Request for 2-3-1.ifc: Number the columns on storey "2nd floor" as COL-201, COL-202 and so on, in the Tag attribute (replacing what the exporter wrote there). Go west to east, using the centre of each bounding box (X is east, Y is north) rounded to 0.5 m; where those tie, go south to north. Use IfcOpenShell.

First a look at what the model holds.

```python
import ifcopenshell
import ifcopenshell.util.element
import ifcopenshell.util.placement

model = ifcopenshell.open("2-3-1.ifc")
print(model.schema)
storey = next(s for s in model.by_type("IfcBuildingStorey") if s.Name == "2nd floor")
columns = [e for e in ifcopenshell.util.element.get_decomposition(storey) if e.is_a("IfcColumn")]
for e in sorted(columns, key=lambda e: e.id()):
    origin = ifcopenshell.util.placement.get_local_placement(e.ObjectPlacement)[:3, 3]
    print(e.id(), e.Tag, e.Name, origin.round(2) + 0.0, sep=" | ")
```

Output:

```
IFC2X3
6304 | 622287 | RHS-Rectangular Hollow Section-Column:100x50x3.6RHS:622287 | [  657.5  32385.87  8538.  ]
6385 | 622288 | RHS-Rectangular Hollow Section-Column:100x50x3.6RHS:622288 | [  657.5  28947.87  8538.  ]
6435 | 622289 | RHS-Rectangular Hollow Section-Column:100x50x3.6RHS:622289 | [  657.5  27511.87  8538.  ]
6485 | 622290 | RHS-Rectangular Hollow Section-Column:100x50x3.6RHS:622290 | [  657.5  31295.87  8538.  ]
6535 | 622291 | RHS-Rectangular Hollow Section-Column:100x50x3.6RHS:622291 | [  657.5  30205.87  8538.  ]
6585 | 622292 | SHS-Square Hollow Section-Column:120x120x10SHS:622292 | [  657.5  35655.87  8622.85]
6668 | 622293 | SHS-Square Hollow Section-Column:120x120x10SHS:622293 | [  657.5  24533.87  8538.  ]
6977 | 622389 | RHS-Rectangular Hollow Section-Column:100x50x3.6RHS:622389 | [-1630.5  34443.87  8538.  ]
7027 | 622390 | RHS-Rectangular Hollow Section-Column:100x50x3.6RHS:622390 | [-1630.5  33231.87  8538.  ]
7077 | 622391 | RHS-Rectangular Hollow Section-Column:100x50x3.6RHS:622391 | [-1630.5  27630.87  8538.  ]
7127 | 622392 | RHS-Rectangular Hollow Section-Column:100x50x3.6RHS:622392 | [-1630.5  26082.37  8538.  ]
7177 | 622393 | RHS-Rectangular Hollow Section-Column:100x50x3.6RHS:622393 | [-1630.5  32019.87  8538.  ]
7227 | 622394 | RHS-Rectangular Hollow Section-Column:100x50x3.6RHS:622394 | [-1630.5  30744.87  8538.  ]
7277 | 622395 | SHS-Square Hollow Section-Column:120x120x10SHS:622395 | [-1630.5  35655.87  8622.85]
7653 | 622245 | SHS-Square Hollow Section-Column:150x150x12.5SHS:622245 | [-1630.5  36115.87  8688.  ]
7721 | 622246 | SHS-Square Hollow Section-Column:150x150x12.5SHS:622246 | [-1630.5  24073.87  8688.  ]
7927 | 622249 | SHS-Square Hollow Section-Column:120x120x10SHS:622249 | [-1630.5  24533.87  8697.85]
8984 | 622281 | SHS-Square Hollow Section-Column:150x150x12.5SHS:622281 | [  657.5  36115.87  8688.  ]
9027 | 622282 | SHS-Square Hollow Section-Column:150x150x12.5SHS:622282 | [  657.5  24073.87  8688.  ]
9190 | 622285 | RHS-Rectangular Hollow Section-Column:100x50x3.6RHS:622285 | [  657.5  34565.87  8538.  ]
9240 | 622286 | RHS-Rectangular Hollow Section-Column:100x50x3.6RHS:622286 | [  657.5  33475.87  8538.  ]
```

```python
import ifcopenshell
import ifcopenshell.geom
import ifcopenshell.util.element
import ifcopenshell.util.shape

model = ifcopenshell.open("2-3-1.ifc")
settings = ifcopenshell.geom.settings()
settings.set("use-world-coords", True)


def centre(element):
    shape = ifcopenshell.geom.create_shape(settings, element)
    return ifcopenshell.util.shape.get_bbox_centroid(shape.geometry)


storey = next(s for s in model.by_type("IfcBuildingStorey") if s.Name == "2nd floor")
columns = [e for e in ifcopenshell.util.element.get_decomposition(storey) if e.is_a("IfcColumn")]

# Insertion points can sit at a corner or the storey origin, so sort by the geometry (in metres).
centres = {e: centre(e) for e in columns}
columns.sort(key=lambda e: (round(centres[e][0] / 0.5), centres[e][1]))

for i, e in enumerate(columns, start=1):
    number = f"COL-2{i:02d}"
    e.Tag = number
    print(e.id(), number)

model.write("2-3-1_v2.ifc")
```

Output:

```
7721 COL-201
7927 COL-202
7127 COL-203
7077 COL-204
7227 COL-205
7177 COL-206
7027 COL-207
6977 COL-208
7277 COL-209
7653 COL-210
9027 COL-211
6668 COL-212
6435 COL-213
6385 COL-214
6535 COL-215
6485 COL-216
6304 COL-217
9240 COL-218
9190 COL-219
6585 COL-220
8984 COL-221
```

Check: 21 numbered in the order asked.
